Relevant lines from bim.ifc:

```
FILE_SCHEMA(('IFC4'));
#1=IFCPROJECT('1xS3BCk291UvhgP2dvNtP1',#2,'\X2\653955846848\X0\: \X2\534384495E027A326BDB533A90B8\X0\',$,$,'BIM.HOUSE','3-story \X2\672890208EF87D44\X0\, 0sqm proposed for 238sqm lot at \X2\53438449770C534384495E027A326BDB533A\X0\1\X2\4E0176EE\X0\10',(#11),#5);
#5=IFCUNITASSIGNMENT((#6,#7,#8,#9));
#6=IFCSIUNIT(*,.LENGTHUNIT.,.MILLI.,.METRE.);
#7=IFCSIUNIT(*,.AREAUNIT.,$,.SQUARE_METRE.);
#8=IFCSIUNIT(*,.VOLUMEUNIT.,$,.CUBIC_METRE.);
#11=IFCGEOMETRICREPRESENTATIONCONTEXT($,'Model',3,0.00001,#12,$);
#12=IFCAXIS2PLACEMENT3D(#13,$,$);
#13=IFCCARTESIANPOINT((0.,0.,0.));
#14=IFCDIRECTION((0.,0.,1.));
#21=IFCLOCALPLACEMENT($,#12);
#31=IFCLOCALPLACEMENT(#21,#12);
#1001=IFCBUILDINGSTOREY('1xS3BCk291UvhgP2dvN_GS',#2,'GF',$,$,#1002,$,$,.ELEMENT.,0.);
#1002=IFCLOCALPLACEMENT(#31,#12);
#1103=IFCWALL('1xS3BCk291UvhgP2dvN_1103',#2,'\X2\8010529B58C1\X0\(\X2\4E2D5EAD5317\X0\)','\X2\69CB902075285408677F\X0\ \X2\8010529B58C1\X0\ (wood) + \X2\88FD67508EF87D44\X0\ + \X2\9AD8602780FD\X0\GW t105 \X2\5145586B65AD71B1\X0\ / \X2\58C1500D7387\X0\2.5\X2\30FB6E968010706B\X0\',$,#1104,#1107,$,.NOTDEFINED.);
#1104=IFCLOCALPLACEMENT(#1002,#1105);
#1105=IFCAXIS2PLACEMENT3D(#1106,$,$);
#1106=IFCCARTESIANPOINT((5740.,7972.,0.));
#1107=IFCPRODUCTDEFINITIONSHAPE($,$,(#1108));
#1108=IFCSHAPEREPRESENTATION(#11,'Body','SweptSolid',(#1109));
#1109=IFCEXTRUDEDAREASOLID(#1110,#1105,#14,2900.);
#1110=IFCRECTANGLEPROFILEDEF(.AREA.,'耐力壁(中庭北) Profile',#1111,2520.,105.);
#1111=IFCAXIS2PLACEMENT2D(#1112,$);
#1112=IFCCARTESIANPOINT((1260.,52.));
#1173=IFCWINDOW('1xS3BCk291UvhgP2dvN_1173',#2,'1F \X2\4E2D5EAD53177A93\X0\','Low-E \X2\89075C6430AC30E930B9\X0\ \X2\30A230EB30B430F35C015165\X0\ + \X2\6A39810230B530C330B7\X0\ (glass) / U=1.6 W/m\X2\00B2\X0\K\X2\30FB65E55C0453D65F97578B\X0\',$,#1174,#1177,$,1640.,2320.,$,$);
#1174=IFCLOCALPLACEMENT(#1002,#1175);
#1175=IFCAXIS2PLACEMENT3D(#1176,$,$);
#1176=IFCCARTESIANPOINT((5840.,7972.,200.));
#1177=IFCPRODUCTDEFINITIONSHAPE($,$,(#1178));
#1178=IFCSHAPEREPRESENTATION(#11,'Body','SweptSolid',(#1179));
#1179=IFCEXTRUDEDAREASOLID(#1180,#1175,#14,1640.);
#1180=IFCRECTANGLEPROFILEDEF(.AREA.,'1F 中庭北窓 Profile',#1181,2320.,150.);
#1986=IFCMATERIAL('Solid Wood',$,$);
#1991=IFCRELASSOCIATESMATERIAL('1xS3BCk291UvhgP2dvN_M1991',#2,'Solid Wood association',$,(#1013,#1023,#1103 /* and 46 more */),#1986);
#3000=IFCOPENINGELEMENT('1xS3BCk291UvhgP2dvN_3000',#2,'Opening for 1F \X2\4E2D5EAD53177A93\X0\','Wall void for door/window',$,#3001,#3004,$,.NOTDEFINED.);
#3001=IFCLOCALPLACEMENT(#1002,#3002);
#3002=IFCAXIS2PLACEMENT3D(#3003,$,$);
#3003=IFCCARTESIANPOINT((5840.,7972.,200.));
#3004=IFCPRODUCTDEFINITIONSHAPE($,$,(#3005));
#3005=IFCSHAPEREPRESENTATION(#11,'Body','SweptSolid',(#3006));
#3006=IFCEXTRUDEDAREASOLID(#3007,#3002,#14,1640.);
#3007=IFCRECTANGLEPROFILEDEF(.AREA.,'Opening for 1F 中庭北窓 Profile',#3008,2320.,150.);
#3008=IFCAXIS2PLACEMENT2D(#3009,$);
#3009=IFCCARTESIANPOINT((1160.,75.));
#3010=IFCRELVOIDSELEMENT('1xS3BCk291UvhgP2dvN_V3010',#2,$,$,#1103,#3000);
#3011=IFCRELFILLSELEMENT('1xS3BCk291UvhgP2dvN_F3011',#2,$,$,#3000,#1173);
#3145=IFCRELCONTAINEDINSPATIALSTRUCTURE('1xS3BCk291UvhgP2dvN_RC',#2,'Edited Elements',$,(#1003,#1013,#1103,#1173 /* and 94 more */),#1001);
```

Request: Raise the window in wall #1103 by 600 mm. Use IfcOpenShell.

```python
import numpy as np
import ifcopenshell
import ifcopenshell.api.geometry
import ifcopenshell.util.placement
import ifcopenshell.util.unit

model = ifcopenshell.open("bim.ifc")
unit_scale = ifcopenshell.util.unit.calculate_unit_scale(model)

window = model.by_guid("1xS3BCk291UvhgP2dvN_1173")
opening = window.FillsVoids[0].RelatingOpeningElement
dz = 600.0

shift = np.array([0.0, 0.0, dz])
# The window is not placed relative to its opening, so move both.
for product in (opening, window):
    matrix = ifcopenshell.util.placement.get_local_placement(product.ObjectPlacement)
    matrix[:3, 3] += shift
    ifcopenshell.api.geometry.edit_object_placement(model, product=product, matrix=matrix, is_si=False)

print(f"moved by {dz * unit_scale:+.3f} m")

model.write("bim_rev.ifc")
```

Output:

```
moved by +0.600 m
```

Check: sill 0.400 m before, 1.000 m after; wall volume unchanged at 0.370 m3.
